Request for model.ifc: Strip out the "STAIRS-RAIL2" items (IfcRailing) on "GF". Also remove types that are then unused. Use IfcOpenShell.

First a look at what the model holds.

```python
import ifcopenshell
import ifcopenshell.util.element

model = ifcopenshell.open("model.ifc")
print(model.schema)
storey = next(s for s in model.by_type("IfcBuildingStorey") if s.Name == "GF")
railings = [e for e in ifcopenshell.util.element.get_decomposition(storey) if e.is_a("IfcRailing")]
seen = {}
for e in railings:
    element_type = ifcopenshell.util.element.get_type(e)
    name = element_type.Name if element_type not in (None, e) else None
    seen[name] = seen.get(name, 0) + 1
for name, count in sorted(seen.items(), key=str):
    print(count, "x", name)
```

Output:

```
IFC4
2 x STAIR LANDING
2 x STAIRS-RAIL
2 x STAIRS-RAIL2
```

```python
import ifcopenshell
import ifcopenshell.api.root
import ifcopenshell.util.element

model = ifcopenshell.open("model.ifc")

storey = next(s for s in model.by_type("IfcBuildingStorey") if s.Name == "GF")
railings = [e for e in ifcopenshell.util.element.get_decomposition(storey) if e.is_a("IfcRailing")]
targets = [e for e in railings if (t := ifcopenshell.util.element.get_type(e)) not in (None, e) and t.Name == "STAIRS-RAIL2"]
types = {ifcopenshell.util.element.get_type(e) for e in targets} - {None, *targets}

for e in targets:
    ifcopenshell.api.root.remove_product(model, product=e)
print(len(targets), "removed")

unused = [t for t in types if not ifcopenshell.util.element.get_types(t)]
for t in unused:
    ifcopenshell.api.root.remove_product(model, product=t)
print(len(unused), "unused types removed")

model.write("model_v2.ifc")
```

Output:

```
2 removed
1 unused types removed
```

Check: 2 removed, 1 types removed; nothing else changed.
